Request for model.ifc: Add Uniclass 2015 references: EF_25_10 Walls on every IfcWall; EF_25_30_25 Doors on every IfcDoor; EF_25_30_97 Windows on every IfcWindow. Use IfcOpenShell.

First a look at what the model holds.

```python
import ifcopenshell

model = ifcopenshell.open("model.ifc")
print(model.schema)
print("classifications:", [c.Name for c in model.by_type("IfcClassification")])
for ifc_class in ("IfcDoor", "IfcRoof", "IfcStair", "IfcWall", "IfcWindow"):
    print(ifc_class, len(model.by_type(ifc_class)))
```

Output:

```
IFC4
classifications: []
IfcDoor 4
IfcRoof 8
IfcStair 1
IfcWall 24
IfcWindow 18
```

```python
import ifcopenshell
import ifcopenshell.api.classification

model = ifcopenshell.open("model.ifc")

system = ifcopenshell.api.classification.add_classification(model, classification="Uniclass 2015")

codes = {
    "IfcWall": ("EF_25_10", "Walls"),
    "IfcDoor": ("EF_25_30_25", "Doors"),
    "IfcWindow": ("EF_25_30_97", "Windows"),
}
for ifc_class, (code, name) in codes.items():
    products = model.by_type(ifc_class)
    ifcopenshell.api.classification.add_reference(
        model, products=products, classification=system, identification=code, name=name
    )
    print(code, len(products))

model.write("model_updated.ifc")
```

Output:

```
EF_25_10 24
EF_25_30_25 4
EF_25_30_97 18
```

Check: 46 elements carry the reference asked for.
